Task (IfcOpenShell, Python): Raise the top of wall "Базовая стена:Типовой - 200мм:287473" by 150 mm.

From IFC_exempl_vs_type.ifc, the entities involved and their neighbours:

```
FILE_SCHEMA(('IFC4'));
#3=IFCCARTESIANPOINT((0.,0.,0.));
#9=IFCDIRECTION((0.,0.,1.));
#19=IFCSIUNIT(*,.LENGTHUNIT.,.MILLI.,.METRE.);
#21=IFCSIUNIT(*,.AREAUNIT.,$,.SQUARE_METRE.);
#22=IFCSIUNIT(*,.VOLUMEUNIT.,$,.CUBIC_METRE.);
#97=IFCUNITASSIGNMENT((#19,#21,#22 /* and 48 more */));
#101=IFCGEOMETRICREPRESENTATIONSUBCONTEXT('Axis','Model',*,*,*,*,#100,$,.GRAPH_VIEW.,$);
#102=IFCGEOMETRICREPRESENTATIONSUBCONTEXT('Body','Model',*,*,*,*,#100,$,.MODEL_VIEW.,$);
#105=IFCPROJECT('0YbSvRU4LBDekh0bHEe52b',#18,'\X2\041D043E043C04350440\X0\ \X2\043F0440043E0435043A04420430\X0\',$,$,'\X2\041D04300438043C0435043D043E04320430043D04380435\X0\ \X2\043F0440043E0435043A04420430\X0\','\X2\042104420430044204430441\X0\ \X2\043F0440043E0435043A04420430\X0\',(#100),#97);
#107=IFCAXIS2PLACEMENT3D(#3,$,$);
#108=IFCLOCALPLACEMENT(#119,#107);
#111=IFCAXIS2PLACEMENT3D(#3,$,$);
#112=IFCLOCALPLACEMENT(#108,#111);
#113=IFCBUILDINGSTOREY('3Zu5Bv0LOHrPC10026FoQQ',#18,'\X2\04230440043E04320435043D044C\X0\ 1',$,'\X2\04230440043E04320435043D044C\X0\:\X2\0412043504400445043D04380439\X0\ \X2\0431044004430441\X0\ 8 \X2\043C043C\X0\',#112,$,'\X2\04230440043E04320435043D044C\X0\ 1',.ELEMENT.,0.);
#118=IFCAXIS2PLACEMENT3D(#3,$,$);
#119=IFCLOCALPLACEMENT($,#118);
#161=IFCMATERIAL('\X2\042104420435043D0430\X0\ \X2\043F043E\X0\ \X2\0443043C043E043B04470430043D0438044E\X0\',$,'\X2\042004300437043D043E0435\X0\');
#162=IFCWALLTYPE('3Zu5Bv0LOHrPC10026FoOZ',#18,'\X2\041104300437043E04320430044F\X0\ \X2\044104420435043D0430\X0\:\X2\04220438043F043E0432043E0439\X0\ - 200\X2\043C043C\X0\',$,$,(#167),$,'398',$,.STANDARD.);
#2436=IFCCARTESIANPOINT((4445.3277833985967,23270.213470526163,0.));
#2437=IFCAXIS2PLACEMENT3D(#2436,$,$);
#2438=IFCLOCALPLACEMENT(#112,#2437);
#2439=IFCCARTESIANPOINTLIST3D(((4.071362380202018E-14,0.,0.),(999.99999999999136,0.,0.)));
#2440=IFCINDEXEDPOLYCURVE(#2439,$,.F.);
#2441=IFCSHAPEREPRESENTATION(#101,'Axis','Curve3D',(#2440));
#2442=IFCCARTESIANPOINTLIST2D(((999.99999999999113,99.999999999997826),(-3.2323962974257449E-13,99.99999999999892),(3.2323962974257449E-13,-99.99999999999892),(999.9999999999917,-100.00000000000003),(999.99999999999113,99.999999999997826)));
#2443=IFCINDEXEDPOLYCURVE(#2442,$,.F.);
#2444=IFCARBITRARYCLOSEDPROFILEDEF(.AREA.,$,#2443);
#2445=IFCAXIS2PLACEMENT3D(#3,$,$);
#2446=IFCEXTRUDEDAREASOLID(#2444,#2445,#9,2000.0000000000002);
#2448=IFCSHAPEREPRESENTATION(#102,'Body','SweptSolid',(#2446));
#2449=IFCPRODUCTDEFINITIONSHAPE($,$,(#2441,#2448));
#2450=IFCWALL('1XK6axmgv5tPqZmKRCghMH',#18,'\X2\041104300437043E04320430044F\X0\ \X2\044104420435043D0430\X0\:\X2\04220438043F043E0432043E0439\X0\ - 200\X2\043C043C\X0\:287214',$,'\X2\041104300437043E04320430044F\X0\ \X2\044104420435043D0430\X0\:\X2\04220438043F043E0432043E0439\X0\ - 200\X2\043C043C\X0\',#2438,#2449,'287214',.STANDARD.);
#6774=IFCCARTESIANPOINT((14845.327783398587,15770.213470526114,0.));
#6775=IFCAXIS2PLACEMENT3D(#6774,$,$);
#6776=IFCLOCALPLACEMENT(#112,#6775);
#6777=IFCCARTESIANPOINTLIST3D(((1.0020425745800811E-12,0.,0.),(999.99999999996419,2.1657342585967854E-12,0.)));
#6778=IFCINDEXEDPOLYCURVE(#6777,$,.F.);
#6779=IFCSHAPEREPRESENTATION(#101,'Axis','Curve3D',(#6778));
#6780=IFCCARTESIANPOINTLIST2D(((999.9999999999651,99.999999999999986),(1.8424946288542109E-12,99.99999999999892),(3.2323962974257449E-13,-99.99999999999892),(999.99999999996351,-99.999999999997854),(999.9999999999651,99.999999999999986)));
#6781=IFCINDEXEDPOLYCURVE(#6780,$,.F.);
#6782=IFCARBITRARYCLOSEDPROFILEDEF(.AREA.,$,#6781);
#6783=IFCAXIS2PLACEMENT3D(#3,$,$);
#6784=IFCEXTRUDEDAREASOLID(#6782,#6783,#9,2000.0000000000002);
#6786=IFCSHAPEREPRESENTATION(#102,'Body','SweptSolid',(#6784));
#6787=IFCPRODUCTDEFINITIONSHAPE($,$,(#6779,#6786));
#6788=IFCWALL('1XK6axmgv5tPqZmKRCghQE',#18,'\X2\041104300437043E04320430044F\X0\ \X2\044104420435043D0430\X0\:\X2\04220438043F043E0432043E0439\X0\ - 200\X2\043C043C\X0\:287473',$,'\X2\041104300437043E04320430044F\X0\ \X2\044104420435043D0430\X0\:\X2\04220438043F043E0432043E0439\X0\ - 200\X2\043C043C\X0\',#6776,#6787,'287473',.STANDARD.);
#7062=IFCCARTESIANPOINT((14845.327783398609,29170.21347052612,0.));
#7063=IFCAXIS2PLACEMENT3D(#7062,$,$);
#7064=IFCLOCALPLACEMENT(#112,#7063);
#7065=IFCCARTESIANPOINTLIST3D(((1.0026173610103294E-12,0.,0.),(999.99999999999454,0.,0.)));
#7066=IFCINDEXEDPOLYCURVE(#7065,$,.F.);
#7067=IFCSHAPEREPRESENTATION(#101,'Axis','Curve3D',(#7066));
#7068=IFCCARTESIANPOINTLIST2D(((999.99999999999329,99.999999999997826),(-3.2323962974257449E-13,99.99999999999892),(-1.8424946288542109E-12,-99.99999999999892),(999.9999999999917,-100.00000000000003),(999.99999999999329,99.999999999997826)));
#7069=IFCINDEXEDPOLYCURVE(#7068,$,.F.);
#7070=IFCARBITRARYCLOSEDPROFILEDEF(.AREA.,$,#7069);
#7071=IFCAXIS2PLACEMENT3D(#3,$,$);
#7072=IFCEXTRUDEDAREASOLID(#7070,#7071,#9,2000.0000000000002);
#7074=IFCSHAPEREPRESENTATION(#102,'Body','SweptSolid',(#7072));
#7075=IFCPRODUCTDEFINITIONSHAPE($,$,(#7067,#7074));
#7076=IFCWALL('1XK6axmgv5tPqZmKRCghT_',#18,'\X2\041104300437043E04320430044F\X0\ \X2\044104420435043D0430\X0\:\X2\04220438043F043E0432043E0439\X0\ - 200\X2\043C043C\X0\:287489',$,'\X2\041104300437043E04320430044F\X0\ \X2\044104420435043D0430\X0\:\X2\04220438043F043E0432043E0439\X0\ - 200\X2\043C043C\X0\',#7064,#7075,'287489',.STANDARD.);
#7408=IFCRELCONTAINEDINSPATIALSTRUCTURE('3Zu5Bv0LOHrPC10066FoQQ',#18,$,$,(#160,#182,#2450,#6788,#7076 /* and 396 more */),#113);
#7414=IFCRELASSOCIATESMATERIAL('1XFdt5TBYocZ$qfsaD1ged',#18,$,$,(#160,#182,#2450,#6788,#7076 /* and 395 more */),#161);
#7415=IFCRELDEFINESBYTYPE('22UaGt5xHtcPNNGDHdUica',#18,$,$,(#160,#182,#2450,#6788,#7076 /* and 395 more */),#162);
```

```python
import ifcopenshell
import ifcopenshell.geom
import ifcopenshell.util.representation
import ifcopenshell.util.shape
import ifcopenshell.util.unit

model = ifcopenshell.open("IFC_exempl_vs_type.ifc")
unit_scale = ifcopenshell.util.unit.calculate_unit_scale(model)
settings = ifcopenshell.geom.settings()


def volume(element):
    """Net volume in cubic metres, openings subtracted."""
    shape = ifcopenshell.geom.create_shape(settings, element)
    return ifcopenshell.util.shape.get_volume(shape.geometry)


wall = model.by_guid("1XK6axmgv5tPqZmKRCghQE")
before = volume(wall)

body = ifcopenshell.util.representation.get_representation(wall, "Model", "Body")
solid = body.Items[0]
old_height = solid.Depth
solid.Depth += 0.15 / unit_scale
after = volume(wall)

print(f"height {old_height:g} -> {solid.Depth:g}, volume {before:.3f} -> {after:.3f} m3")

model.write("IFC_exempl_vs_type-out.ifc")
```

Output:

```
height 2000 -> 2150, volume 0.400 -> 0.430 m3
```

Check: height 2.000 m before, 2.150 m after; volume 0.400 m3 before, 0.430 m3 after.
